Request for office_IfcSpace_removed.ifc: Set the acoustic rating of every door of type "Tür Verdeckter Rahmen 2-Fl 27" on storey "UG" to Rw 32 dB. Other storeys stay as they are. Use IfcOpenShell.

First a look at what the model holds.

```python
import ifcopenshell
import ifcopenshell.util.element

model = ifcopenshell.open("office_IfcSpace_removed.ifc")
print(model.schema)
storey = next(s for s in model.by_type("IfcBuildingStorey") if s.Name == "UG")
doors = [e for e in ifcopenshell.util.element.get_decomposition(storey) if e.is_a("IfcDoor")]
seen = {}
for e in doors:
    element_type = ifcopenshell.util.element.get_type(e)
    key = (element_type.Name if element_type != e and element_type else None, ifcopenshell.util.element.get_pset(e, "Pset_DoorCommon", "AcousticRating"))
    seen[key] = seen.get(key, 0) + 1
for (name, value), count in sorted(seen.items(), key=str):
    print(count, "x", name, "|", value)
```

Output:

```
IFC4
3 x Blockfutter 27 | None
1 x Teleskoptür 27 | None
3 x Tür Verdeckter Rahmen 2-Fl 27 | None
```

```python
import ifcopenshell
import ifcopenshell.api.pset
import ifcopenshell.util.element

model = ifcopenshell.open("office_IfcSpace_removed.ifc")

storey = next(s for s in model.by_type("IfcBuildingStorey") if s.Name == "UG")
doors = [e for e in ifcopenshell.util.element.get_decomposition(storey) if e.is_a("IfcDoor")]

count = 0
for e in doors:
    element_type = ifcopenshell.util.element.get_type(e)
    if element_type in (None, e) or element_type.Name != "Tür Verdeckter Rahmen 2-Fl 27":
        continue
    # add_pset returns the element's existing set when there is one.
    pset = ifcopenshell.api.pset.add_pset(model, product=e, name="Pset_DoorCommon")
    ifcopenshell.api.pset.edit_pset(model, pset=pset, properties={"AcousticRating": "Rw 32 dB"})
    count += 1

print(count, "doors updated")

model.write("office_IfcSpace_removed_updated.ifc")
```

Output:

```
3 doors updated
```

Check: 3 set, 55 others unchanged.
